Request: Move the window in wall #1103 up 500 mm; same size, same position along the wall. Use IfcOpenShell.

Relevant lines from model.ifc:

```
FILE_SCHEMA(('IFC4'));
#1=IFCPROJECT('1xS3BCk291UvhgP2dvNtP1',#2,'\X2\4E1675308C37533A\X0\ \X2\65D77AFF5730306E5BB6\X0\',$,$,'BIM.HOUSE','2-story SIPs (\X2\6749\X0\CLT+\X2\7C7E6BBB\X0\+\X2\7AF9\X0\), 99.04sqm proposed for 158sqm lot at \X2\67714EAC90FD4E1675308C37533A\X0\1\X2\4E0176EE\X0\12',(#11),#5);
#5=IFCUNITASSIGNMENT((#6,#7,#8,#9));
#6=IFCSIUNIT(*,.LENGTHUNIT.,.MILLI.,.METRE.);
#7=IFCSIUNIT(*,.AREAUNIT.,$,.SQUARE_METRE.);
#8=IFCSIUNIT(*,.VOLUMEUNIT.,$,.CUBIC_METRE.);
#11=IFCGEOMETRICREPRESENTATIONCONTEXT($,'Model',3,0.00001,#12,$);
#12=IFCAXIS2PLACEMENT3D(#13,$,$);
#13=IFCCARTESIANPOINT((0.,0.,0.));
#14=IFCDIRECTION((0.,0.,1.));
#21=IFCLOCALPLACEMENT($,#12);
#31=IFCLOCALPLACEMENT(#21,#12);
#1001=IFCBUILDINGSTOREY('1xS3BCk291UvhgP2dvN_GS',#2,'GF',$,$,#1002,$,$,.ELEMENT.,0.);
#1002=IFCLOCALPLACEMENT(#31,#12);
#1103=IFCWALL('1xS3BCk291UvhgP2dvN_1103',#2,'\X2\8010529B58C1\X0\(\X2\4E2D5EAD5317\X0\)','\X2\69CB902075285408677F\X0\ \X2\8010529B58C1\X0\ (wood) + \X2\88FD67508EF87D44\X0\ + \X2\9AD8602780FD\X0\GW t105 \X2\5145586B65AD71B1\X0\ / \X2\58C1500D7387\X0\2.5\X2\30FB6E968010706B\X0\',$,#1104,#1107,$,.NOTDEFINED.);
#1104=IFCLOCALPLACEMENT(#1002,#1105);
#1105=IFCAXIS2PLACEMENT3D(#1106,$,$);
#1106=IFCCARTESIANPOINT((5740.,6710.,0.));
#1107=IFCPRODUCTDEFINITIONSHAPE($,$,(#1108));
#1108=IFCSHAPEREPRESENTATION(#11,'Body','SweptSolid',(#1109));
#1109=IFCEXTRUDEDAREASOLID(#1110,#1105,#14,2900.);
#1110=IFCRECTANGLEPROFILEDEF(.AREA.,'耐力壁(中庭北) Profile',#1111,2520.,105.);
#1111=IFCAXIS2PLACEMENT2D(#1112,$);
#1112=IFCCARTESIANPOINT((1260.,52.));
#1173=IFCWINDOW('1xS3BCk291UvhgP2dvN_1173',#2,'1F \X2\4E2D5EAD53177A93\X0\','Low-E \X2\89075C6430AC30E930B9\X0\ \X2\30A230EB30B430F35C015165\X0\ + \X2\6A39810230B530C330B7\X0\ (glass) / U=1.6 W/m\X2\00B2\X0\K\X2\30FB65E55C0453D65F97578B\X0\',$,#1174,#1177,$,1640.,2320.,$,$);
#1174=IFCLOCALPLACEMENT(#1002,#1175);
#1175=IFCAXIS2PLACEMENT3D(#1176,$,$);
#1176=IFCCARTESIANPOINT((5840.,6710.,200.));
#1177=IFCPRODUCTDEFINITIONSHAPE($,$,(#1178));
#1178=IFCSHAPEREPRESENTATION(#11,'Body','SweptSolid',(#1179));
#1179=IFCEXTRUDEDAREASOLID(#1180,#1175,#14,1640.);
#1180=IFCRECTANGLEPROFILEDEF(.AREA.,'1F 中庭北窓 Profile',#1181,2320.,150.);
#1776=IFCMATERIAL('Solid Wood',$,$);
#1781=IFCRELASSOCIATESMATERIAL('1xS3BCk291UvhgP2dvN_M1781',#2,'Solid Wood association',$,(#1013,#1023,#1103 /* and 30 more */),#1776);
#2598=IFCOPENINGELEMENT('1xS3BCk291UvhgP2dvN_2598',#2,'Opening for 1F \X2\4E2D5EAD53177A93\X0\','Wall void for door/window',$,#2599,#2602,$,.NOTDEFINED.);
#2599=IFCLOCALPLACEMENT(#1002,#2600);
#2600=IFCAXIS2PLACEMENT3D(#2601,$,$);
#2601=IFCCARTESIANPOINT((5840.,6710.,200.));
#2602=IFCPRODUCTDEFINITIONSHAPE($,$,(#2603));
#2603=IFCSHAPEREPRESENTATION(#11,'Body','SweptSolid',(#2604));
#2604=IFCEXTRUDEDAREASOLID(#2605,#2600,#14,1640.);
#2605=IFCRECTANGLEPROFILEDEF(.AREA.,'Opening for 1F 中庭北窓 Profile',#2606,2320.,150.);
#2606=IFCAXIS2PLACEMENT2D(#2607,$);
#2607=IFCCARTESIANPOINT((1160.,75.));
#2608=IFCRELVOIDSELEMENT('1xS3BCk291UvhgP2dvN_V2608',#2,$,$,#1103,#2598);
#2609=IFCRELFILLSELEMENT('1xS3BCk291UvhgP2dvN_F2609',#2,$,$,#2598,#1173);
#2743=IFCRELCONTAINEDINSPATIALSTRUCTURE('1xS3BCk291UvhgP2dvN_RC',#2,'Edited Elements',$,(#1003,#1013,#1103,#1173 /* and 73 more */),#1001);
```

```python
import numpy as np
import ifcopenshell
import ifcopenshell.api.geometry
import ifcopenshell.util.placement
import ifcopenshell.util.unit

model = ifcopenshell.open("model.ifc")
unit_scale = ifcopenshell.util.unit.calculate_unit_scale(model)

window = model.by_guid("1xS3BCk291UvhgP2dvN_1173")
opening = window.FillsVoids[0].RelatingOpeningElement
dz = 0.5 / unit_scale

shift = np.array([0.0, 0.0, dz])
# The window is not placed relative to its opening, so move both.
for product in (opening, window):
    matrix = ifcopenshell.util.placement.get_local_placement(product.ObjectPlacement)
    matrix[:3, 3] += shift
    ifcopenshell.api.geometry.edit_object_placement(model, product=product, matrix=matrix, is_si=False)

print(f"moved by {dz * unit_scale:+.3f} m")

model.write("model_updated.ifc")
```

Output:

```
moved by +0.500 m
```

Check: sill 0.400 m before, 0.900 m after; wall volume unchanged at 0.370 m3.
